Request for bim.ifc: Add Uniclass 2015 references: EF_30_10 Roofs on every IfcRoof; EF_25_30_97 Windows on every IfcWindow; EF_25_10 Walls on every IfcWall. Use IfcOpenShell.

First a look at what the model holds.

```python
import ifcopenshell

model = ifcopenshell.open("bim.ifc")
print(model.schema)
print("classifications:", [c.Name for c in model.by_type("IfcClassification")])
for ifc_class in ("IfcDoor", "IfcRoof", "IfcStair", "IfcWall", "IfcWindow"):
    print(ifc_class, len(model.by_type(ifc_class)))
```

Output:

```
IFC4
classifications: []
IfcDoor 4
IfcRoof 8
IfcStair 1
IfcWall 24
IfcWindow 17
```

```python
import ifcopenshell
import ifcopenshell.api.classification

model = ifcopenshell.open("bim.ifc")

system = ifcopenshell.api.classification.add_classification(model, classification="Uniclass 2015")

codes = {
    "IfcRoof": ("EF_30_10", "Roofs"),
    "IfcWindow": ("EF_25_30_97", "Windows"),
    "IfcWall": ("EF_25_10", "Walls"),
}
for ifc_class, (code, name) in codes.items():
    products = model.by_type(ifc_class)
    ifcopenshell.api.classification.add_reference(
        model, products=products, classification=system, identification=code, name=name
    )
    print(code, len(products))

model.write("bim_rev.ifc")
```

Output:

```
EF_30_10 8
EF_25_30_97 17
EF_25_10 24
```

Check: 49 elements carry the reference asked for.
